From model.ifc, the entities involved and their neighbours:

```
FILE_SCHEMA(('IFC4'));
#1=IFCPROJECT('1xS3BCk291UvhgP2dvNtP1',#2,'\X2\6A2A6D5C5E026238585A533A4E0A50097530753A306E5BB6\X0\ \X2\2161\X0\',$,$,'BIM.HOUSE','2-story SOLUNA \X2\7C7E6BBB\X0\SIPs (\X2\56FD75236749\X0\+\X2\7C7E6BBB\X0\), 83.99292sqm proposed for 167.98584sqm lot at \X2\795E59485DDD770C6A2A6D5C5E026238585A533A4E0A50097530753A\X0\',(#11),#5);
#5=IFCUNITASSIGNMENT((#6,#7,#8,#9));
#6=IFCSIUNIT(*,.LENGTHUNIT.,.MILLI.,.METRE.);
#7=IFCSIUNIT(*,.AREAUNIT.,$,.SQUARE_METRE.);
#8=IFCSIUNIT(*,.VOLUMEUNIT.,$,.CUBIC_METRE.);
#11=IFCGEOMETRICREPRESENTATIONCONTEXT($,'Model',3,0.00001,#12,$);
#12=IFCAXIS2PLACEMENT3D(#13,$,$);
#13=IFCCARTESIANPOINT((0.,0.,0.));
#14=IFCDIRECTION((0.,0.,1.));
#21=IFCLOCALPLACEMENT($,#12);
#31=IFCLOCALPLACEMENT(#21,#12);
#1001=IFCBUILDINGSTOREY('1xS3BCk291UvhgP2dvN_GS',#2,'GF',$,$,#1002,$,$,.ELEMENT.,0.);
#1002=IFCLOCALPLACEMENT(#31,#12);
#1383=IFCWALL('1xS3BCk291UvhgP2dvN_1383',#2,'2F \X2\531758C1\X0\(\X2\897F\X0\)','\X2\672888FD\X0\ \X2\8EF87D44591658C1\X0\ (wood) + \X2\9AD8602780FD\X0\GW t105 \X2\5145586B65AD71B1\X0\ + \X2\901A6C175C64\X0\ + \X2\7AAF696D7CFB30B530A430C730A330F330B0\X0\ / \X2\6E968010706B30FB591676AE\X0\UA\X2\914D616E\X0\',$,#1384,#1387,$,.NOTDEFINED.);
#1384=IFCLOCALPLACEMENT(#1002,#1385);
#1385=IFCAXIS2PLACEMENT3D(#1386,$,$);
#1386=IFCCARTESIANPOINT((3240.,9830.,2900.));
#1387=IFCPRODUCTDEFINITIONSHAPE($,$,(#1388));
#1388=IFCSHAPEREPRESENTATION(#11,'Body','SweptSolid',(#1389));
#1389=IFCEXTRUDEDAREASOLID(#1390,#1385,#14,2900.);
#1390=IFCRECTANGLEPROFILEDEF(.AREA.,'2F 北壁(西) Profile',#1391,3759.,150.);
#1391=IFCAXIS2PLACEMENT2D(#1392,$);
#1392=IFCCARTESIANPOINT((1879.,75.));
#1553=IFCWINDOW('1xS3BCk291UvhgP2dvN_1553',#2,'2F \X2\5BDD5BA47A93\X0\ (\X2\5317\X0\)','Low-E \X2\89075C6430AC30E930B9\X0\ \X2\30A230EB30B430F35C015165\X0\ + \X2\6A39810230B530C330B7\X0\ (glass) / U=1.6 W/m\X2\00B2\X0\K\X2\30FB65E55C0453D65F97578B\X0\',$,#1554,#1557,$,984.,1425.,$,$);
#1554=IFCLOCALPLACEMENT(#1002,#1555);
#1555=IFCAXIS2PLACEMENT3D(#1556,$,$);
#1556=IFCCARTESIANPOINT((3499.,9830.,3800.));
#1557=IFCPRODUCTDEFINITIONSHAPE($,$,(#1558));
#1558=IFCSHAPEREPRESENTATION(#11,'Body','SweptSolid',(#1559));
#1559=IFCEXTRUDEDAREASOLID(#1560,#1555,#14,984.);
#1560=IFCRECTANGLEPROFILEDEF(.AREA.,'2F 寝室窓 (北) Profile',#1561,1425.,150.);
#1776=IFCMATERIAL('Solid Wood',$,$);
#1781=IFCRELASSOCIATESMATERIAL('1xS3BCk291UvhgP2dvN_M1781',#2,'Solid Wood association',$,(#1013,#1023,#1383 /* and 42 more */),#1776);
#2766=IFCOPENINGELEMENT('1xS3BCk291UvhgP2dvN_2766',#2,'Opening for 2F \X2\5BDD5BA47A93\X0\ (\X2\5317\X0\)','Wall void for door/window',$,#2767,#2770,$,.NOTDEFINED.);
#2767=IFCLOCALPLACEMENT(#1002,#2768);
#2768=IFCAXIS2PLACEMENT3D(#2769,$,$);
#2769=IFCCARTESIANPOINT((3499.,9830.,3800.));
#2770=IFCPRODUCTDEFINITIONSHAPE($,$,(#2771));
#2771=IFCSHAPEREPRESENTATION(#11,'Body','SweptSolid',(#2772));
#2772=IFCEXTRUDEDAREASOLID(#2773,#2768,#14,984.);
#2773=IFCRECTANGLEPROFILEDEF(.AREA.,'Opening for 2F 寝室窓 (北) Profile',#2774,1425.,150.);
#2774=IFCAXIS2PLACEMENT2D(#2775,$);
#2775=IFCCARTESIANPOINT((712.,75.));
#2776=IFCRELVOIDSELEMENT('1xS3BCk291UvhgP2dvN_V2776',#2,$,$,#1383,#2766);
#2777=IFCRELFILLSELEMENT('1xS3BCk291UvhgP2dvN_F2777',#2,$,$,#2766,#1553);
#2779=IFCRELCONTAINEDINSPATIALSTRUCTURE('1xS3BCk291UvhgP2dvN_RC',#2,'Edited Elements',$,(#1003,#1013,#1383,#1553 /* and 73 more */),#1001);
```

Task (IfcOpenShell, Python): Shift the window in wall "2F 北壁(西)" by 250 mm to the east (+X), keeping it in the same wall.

```python
import ifcopenshell
import ifcopenshell.api.geometry
import ifcopenshell.util.placement
import ifcopenshell.util.unit

model = ifcopenshell.open("model.ifc")
unit_scale = ifcopenshell.util.unit.calculate_unit_scale(model)

window = model.by_guid("1xS3BCk291UvhgP2dvN_1553")
opening = window.FillsVoids[0].RelatingOpeningElement
wall = opening.VoidsElements[0].RelatingBuildingElement

wall_matrix = ifcopenshell.util.placement.get_local_placement(wall.ObjectPlacement)
shift = wall_matrix[:3, 0] * 0.25 / unit_scale
before = ifcopenshell.util.placement.get_local_placement(window.ObjectPlacement)[:3, 3].copy()

# The window is not placed relative to its opening, so move both.
for product in (opening, window):
    matrix = ifcopenshell.util.placement.get_local_placement(product.ObjectPlacement)
    matrix[:3, 3] += shift
    ifcopenshell.api.geometry.edit_object_placement(model, product=product, matrix=matrix, is_si=False)

after = ifcopenshell.util.placement.get_local_placement(window.ObjectPlacement)[:3, 3]
print("window moved by", (after - before).round(3) + 0.0)

model.write("model_edited.ifc")
```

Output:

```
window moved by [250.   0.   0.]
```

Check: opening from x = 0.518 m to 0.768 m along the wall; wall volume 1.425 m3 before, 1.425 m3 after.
